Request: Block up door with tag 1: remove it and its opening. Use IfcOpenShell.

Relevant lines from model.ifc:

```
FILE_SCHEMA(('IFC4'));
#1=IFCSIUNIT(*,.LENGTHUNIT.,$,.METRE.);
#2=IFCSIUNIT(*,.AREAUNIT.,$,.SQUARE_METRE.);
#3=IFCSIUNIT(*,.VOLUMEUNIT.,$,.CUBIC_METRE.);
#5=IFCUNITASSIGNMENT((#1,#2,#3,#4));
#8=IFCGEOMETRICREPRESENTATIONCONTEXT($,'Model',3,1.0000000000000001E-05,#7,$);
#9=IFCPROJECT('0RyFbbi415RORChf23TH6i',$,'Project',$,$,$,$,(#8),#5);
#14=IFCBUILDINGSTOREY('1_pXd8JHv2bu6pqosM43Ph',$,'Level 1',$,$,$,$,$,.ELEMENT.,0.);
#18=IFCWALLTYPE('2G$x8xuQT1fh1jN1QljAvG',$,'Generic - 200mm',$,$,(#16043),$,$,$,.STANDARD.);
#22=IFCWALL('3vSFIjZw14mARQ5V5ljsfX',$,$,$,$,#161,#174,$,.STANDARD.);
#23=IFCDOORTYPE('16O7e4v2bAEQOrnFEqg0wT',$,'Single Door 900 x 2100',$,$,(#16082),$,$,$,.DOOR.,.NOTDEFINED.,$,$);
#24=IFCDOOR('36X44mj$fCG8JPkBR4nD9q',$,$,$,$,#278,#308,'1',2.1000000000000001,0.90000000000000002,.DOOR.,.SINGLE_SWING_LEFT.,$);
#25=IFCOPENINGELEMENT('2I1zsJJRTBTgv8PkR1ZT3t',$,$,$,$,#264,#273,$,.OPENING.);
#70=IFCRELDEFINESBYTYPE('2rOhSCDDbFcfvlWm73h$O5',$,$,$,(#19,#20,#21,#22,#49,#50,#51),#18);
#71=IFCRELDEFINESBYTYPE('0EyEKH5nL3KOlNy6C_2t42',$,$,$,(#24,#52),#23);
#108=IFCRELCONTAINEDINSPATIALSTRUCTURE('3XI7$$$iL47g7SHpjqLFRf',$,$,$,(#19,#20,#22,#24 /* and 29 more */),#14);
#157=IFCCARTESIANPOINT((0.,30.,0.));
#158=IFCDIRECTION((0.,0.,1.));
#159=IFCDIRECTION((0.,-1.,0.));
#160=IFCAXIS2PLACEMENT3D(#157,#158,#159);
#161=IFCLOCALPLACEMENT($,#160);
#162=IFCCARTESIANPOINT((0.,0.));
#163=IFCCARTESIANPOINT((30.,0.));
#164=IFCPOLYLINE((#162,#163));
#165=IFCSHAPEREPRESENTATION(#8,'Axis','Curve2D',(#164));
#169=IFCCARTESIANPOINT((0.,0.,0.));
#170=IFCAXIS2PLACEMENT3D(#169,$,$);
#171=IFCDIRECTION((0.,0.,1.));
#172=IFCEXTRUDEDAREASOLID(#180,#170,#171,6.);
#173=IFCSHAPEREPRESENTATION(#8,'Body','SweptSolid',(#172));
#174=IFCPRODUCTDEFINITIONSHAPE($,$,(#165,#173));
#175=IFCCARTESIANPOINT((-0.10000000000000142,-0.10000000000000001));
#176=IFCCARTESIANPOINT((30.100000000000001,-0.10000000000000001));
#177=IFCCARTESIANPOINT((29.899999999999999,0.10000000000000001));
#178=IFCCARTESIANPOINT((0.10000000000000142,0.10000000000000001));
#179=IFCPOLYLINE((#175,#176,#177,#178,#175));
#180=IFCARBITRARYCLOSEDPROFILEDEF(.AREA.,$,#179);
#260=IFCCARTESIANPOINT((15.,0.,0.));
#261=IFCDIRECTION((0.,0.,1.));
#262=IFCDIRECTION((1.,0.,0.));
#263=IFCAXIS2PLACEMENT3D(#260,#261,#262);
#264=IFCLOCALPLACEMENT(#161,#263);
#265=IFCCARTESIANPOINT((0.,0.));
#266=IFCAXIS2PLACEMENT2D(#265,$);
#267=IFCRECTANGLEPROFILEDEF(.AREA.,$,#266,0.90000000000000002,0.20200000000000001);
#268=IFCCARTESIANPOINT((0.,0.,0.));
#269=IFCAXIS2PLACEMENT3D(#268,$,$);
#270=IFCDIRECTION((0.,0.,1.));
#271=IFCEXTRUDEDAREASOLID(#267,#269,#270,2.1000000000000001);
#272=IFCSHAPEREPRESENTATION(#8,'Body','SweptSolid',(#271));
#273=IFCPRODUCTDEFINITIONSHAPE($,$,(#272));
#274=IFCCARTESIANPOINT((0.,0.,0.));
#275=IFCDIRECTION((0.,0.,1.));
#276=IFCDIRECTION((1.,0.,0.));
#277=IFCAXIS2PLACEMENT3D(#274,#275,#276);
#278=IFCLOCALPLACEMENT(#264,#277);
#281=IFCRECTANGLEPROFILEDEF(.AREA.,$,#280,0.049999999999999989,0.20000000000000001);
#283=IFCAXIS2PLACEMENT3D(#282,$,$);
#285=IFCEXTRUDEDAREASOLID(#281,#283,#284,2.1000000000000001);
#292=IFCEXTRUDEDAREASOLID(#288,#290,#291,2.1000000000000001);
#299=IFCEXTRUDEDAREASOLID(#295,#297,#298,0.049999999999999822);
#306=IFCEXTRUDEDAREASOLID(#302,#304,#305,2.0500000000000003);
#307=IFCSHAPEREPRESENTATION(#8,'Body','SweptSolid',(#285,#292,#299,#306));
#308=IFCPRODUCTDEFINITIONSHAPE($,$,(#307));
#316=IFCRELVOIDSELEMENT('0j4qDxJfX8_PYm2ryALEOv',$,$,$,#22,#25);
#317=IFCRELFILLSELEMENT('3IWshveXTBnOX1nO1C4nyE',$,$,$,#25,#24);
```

```python
import ifcopenshell
import ifcopenshell.api.feature
import ifcopenshell.api.root
import ifcopenshell.geom
import ifcopenshell.util.shape

model = ifcopenshell.open("model.ifc")
settings = ifcopenshell.geom.settings()


def volume(element):
    """Net volume in cubic metres, openings subtracted."""
    shape = ifcopenshell.geom.create_shape(settings, element)
    return ifcopenshell.util.shape.get_volume(shape.geometry)


door = model.by_guid("36X44mj$fCG8JPkBR4nD9q")
opening = door.FillsVoids[0].RelatingOpeningElement
wall = opening.VoidsElements[0].RelatingBuildingElement
before = volume(wall)

ifcopenshell.api.root.remove_product(model, product=door)
ifcopenshell.api.feature.remove_feature(model, feature=opening)

after = volume(wall)

print(f"wall volume {before:.3f} -> {after:.3f} m3")

model.write("model_updated.ifc")
```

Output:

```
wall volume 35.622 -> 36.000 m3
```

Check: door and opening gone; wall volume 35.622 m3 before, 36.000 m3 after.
